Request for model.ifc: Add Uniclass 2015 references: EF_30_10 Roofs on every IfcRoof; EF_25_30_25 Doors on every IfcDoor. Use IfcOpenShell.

First a look at what the model holds.

```python
import ifcopenshell

model = ifcopenshell.open("model.ifc")
print(model.schema)
print("classifications:", [c.Name for c in model.by_type("IfcClassification")])
for ifc_class in ("IfcDoor", "IfcRoof", "IfcStair", "IfcWall", "IfcWindow"):
    print(ifc_class, len(model.by_type(ifc_class)))
```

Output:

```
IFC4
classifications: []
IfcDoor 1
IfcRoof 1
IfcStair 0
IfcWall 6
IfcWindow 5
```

```python
import ifcopenshell
import ifcopenshell.api.classification

model = ifcopenshell.open("model.ifc")

system = ifcopenshell.api.classification.add_classification(model, classification="Uniclass 2015")

codes = {
    "IfcRoof": ("EF_30_10", "Roofs"),
    "IfcDoor": ("EF_25_30_25", "Doors"),
}
for ifc_class, (code, name) in codes.items():
    products = model.by_type(ifc_class)
    ifcopenshell.api.classification.add_reference(
        model, products=products, classification=system, identification=code, name=name
    )
    print(code, len(products))

model.write("model_v2.ifc")
```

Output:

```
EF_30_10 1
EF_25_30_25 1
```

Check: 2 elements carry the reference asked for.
